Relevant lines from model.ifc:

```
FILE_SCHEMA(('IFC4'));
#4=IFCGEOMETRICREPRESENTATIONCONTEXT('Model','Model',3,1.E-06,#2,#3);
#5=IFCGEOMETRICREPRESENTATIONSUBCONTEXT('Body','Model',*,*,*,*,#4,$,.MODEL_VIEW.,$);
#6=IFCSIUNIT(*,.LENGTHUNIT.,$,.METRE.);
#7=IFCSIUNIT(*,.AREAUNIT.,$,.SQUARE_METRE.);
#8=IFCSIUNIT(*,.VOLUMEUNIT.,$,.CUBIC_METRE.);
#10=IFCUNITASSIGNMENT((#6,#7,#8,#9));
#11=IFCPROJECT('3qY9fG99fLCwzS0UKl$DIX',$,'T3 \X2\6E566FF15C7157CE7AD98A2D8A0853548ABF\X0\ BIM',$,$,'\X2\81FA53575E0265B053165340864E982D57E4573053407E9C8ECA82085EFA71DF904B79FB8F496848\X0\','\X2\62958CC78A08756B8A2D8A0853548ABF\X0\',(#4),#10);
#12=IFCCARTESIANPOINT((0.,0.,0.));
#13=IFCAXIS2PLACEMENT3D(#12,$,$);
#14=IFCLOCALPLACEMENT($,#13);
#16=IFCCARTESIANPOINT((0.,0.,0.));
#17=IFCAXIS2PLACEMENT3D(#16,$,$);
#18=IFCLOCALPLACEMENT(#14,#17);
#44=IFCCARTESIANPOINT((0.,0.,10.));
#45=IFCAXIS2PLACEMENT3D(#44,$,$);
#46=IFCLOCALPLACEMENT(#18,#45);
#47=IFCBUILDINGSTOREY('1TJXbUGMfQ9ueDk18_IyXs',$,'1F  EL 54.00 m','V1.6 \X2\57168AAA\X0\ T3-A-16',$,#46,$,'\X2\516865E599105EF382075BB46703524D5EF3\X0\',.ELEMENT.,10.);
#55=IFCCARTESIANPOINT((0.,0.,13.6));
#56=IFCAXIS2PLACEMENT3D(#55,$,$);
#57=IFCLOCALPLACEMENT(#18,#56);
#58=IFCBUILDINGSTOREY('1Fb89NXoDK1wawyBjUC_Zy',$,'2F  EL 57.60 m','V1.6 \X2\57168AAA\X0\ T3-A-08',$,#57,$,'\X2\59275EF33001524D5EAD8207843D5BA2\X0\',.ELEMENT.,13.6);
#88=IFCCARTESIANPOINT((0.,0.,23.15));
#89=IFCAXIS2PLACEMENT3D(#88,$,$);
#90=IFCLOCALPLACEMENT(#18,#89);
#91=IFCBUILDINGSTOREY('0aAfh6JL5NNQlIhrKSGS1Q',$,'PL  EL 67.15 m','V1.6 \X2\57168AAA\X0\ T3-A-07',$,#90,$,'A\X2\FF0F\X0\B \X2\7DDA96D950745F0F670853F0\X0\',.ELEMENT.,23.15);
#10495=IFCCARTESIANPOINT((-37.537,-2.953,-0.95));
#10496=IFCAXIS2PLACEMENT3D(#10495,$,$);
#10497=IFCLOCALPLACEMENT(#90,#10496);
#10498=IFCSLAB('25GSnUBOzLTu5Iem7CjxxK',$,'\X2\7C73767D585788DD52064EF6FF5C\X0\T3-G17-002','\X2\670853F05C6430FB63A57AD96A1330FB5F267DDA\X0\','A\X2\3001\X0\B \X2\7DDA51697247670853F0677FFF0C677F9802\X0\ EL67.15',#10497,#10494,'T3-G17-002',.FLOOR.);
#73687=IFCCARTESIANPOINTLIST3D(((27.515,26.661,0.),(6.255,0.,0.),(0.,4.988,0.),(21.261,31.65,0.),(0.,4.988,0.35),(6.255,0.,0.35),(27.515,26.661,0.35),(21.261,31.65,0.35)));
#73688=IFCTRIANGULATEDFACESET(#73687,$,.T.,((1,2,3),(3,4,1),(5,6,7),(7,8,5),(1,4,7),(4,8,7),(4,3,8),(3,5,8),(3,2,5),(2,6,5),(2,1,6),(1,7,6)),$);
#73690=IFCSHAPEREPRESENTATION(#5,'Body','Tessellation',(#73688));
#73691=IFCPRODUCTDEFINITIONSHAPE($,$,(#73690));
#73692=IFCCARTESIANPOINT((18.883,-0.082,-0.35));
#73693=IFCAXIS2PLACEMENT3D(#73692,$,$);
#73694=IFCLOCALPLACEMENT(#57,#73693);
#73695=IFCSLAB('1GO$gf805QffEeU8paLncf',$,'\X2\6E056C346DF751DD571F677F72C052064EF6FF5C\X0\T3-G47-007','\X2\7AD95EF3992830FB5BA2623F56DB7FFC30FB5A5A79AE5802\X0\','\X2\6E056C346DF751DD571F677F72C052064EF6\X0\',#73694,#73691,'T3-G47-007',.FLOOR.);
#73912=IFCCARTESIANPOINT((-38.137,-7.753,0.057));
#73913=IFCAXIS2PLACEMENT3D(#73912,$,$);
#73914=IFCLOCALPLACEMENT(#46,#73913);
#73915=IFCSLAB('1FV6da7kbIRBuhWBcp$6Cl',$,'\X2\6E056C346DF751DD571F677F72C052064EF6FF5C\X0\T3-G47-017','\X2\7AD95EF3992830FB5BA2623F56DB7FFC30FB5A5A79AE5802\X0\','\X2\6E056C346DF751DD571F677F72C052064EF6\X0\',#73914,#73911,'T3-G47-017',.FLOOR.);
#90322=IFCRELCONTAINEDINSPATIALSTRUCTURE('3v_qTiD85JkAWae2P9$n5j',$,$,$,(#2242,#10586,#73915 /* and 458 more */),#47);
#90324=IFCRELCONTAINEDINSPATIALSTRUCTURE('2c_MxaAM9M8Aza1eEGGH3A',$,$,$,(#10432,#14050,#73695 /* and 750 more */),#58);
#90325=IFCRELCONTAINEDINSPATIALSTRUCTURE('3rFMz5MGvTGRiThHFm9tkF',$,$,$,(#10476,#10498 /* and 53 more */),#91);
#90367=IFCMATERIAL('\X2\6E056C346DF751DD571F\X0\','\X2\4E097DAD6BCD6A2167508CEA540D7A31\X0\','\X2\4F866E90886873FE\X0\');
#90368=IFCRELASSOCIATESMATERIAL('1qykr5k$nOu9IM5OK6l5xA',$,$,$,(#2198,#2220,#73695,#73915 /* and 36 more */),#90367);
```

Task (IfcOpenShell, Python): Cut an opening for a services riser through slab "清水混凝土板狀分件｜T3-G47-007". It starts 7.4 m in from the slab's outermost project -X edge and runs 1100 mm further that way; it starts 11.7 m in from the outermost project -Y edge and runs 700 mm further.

```python
import numpy as np
import ifcopenshell
import ifcopenshell.api.feature
import ifcopenshell.api.geometry
import ifcopenshell.api.root
import ifcopenshell.geom
import ifcopenshell.util.placement
import ifcopenshell.util.representation
import ifcopenshell.util.shape
import ifcopenshell.util.unit

model = ifcopenshell.open("model.ifc")
unit_scale = ifcopenshell.util.unit.calculate_unit_scale(model)
settings = ifcopenshell.geom.settings()


def volume(element):
    """Net volume in cubic metres, openings subtracted."""
    shape = ifcopenshell.geom.create_shape(settings, element)
    return ifcopenshell.util.shape.get_volume(shape.geometry)


slab = model.by_guid("1GO$gf805QffEeU8paLncf")
before = volume(slab)

# Extent in the slab's own axes, in metres. The edges named are its -X and -Y sides.
slab_shape = ifcopenshell.geom.create_shape(settings, slab)
vertices = ifcopenshell.util.shape.get_vertices(slab_shape.geometry)
x_min, y_min, bottom = vertices.min(axis=0)
top = vertices[:, 2].max()

opening = ifcopenshell.api.root.create_entity(model, ifc_class="IfcOpeningElement", name="Services riser opening", predefined_type="OPENING")
context = ifcopenshell.util.representation.get_context(model, "Model", "Body", "MODEL_VIEW")
width, depth = 1.1, 0.7
outline = [(0.0, 0.0), (width, 0.0), (width, depth), (0.0, depth), (0.0, 0.0)]
# Overshoot both faces by 50 mm so the cut is clean.
shape = ifcopenshell.api.geometry.add_slab_representation(
    model, context=context, depth=top - bottom + 0.1, polyline=outline
)
ifcopenshell.api.geometry.assign_representation(model, product=opening, representation=shape)

matrix = ifcopenshell.util.placement.get_local_placement(slab.ObjectPlacement)
matrix[:, 3] = matrix @ np.append(np.array([x_min + 7.4, y_min + 11.7, bottom - 0.05]) / unit_scale, 1.0)
ifcopenshell.api.geometry.edit_object_placement(model, product=opening, matrix=matrix, is_si=False)
ifcopenshell.api.feature.add_feature(model, feature=opening, element=slab)

after = volume(slab)

print(f"slab volume {before:.3f} -> {after:.3f} m3")

model.write("model-out.ifc")
```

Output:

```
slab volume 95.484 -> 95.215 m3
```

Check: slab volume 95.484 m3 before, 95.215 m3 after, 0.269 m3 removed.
